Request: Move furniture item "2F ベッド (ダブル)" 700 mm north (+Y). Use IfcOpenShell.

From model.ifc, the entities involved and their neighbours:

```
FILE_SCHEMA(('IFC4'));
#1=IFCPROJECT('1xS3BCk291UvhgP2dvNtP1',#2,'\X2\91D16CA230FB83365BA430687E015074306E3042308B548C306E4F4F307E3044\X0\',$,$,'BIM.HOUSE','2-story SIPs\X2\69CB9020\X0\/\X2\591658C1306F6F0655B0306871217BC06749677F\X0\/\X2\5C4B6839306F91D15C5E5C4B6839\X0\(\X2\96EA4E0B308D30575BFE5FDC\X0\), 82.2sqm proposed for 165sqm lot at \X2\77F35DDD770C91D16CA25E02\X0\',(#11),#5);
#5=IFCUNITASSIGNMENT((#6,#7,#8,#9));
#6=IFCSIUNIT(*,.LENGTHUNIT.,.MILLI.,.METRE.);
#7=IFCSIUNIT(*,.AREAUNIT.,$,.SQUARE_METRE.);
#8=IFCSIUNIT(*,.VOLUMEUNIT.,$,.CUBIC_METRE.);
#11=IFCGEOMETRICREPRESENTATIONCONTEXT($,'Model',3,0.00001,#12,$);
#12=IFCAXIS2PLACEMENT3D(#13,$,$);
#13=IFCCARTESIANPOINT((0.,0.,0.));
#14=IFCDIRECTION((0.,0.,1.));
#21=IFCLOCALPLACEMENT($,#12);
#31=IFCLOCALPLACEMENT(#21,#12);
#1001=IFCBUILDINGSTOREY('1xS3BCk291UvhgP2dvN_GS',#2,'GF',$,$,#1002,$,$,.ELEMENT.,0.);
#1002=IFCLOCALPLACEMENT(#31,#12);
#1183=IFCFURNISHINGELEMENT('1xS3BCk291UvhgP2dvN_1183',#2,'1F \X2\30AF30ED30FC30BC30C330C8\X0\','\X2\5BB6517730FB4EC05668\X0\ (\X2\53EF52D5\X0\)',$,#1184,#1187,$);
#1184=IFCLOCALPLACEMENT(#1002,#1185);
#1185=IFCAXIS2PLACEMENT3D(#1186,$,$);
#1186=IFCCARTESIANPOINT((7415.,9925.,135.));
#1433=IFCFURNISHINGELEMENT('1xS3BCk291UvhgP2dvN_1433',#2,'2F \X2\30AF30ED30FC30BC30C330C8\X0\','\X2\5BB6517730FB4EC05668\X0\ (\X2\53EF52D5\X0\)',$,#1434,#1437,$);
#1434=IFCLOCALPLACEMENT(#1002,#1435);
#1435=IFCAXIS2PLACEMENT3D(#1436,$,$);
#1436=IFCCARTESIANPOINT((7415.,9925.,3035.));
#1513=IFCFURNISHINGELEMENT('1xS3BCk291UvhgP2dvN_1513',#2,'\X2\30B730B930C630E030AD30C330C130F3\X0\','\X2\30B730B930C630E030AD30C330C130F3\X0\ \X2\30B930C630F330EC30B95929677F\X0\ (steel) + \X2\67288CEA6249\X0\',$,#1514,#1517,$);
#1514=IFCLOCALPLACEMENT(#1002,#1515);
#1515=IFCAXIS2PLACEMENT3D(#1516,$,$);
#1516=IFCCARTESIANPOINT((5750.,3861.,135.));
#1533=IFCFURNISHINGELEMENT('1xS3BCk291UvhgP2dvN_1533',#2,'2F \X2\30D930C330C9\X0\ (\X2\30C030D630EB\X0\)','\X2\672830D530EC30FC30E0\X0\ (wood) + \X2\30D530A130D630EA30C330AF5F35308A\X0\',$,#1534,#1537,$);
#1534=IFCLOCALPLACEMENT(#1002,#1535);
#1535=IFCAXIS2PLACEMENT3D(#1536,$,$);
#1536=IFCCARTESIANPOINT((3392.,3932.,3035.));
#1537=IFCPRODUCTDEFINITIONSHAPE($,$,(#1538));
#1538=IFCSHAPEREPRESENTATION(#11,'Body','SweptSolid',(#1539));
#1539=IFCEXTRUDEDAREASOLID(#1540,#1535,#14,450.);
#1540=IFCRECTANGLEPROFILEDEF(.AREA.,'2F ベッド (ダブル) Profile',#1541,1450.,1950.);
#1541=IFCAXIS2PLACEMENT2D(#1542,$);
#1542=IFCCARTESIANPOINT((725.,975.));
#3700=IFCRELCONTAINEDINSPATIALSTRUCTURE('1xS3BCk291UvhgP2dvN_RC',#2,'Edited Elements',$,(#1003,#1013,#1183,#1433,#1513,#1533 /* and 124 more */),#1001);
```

```python
import ifcopenshell
import ifcopenshell.api.geometry
import ifcopenshell.util.placement

model = ifcopenshell.open("model.ifc")

item = model.by_guid("1xS3BCk291UvhgP2dvN_1533")
matrix = ifcopenshell.util.placement.get_local_placement(item.ObjectPlacement)
matrix[1, 3] += 700.0
ifcopenshell.api.geometry.edit_object_placement(model, product=item, matrix=matrix, is_si=False)

print(ifcopenshell.util.placement.get_local_placement(item.ObjectPlacement).round(3) + 0.0)

model.write("model_v2.ifc")
```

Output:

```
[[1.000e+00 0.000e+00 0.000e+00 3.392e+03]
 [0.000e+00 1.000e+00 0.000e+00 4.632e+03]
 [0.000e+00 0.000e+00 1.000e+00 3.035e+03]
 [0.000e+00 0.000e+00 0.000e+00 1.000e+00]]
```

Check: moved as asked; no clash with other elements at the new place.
